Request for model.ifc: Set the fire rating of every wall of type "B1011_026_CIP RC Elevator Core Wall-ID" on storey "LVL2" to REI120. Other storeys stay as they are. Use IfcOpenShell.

First a look at what the model holds.

```python
import ifcopenshell
import ifcopenshell.util.element

model = ifcopenshell.open("model.ifc")
print(model.schema)
storey = next(s for s in model.by_type("IfcBuildingStorey") if s.Name == "LVL2")
walls = [e for e in ifcopenshell.util.element.get_decomposition(storey) if e.is_a("IfcWall")]
seen = {}
for e in walls:
    element_type = ifcopenshell.util.element.get_type(e)
    key = (element_type.Name if element_type != e and element_type else None, ifcopenshell.util.element.get_pset(e, "Pset_WallCommon", "FireRating"))
    seen[key] = seen.get(key, 0) + 1
for (name, value), count in sorted(seen.items(), key=str):
    print(count, "x", name, "|", value)
```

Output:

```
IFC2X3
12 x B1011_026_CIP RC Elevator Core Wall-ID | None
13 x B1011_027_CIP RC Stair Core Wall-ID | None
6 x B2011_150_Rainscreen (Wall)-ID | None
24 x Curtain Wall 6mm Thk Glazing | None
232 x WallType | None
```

```python
import ifcopenshell
import ifcopenshell.api.pset
import ifcopenshell.util.element

model = ifcopenshell.open("model.ifc")

storey = next(s for s in model.by_type("IfcBuildingStorey") if s.Name == "LVL2")
walls = [e for e in ifcopenshell.util.element.get_decomposition(storey) if e.is_a("IfcWall")]

count = 0
for e in walls:
    element_type = ifcopenshell.util.element.get_type(e)
    if element_type in (None, e) or element_type.Name != "B1011_026_CIP RC Elevator Core Wall-ID":
        continue
    found = ifcopenshell.util.element.get_pset(e, "Pset_WallCommon", should_inherit=False)
    if found:
        pset = model.by_id(found["id"])
        if len(ifcopenshell.util.element.get_elements_by_pset(pset)) > 1:
            pset = ifcopenshell.api.pset.unshare_pset(model, products=[e], pset=pset)[0]
    else:
        pset = ifcopenshell.api.pset.add_pset(model, product=e, name="Pset_WallCommon")
    ifcopenshell.api.pset.edit_pset(model, pset=pset, properties={"FireRating": "REI120"})
    count += 1

print(count, "walls updated")

model.write("model_rev.ifc")
```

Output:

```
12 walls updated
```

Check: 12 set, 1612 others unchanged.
